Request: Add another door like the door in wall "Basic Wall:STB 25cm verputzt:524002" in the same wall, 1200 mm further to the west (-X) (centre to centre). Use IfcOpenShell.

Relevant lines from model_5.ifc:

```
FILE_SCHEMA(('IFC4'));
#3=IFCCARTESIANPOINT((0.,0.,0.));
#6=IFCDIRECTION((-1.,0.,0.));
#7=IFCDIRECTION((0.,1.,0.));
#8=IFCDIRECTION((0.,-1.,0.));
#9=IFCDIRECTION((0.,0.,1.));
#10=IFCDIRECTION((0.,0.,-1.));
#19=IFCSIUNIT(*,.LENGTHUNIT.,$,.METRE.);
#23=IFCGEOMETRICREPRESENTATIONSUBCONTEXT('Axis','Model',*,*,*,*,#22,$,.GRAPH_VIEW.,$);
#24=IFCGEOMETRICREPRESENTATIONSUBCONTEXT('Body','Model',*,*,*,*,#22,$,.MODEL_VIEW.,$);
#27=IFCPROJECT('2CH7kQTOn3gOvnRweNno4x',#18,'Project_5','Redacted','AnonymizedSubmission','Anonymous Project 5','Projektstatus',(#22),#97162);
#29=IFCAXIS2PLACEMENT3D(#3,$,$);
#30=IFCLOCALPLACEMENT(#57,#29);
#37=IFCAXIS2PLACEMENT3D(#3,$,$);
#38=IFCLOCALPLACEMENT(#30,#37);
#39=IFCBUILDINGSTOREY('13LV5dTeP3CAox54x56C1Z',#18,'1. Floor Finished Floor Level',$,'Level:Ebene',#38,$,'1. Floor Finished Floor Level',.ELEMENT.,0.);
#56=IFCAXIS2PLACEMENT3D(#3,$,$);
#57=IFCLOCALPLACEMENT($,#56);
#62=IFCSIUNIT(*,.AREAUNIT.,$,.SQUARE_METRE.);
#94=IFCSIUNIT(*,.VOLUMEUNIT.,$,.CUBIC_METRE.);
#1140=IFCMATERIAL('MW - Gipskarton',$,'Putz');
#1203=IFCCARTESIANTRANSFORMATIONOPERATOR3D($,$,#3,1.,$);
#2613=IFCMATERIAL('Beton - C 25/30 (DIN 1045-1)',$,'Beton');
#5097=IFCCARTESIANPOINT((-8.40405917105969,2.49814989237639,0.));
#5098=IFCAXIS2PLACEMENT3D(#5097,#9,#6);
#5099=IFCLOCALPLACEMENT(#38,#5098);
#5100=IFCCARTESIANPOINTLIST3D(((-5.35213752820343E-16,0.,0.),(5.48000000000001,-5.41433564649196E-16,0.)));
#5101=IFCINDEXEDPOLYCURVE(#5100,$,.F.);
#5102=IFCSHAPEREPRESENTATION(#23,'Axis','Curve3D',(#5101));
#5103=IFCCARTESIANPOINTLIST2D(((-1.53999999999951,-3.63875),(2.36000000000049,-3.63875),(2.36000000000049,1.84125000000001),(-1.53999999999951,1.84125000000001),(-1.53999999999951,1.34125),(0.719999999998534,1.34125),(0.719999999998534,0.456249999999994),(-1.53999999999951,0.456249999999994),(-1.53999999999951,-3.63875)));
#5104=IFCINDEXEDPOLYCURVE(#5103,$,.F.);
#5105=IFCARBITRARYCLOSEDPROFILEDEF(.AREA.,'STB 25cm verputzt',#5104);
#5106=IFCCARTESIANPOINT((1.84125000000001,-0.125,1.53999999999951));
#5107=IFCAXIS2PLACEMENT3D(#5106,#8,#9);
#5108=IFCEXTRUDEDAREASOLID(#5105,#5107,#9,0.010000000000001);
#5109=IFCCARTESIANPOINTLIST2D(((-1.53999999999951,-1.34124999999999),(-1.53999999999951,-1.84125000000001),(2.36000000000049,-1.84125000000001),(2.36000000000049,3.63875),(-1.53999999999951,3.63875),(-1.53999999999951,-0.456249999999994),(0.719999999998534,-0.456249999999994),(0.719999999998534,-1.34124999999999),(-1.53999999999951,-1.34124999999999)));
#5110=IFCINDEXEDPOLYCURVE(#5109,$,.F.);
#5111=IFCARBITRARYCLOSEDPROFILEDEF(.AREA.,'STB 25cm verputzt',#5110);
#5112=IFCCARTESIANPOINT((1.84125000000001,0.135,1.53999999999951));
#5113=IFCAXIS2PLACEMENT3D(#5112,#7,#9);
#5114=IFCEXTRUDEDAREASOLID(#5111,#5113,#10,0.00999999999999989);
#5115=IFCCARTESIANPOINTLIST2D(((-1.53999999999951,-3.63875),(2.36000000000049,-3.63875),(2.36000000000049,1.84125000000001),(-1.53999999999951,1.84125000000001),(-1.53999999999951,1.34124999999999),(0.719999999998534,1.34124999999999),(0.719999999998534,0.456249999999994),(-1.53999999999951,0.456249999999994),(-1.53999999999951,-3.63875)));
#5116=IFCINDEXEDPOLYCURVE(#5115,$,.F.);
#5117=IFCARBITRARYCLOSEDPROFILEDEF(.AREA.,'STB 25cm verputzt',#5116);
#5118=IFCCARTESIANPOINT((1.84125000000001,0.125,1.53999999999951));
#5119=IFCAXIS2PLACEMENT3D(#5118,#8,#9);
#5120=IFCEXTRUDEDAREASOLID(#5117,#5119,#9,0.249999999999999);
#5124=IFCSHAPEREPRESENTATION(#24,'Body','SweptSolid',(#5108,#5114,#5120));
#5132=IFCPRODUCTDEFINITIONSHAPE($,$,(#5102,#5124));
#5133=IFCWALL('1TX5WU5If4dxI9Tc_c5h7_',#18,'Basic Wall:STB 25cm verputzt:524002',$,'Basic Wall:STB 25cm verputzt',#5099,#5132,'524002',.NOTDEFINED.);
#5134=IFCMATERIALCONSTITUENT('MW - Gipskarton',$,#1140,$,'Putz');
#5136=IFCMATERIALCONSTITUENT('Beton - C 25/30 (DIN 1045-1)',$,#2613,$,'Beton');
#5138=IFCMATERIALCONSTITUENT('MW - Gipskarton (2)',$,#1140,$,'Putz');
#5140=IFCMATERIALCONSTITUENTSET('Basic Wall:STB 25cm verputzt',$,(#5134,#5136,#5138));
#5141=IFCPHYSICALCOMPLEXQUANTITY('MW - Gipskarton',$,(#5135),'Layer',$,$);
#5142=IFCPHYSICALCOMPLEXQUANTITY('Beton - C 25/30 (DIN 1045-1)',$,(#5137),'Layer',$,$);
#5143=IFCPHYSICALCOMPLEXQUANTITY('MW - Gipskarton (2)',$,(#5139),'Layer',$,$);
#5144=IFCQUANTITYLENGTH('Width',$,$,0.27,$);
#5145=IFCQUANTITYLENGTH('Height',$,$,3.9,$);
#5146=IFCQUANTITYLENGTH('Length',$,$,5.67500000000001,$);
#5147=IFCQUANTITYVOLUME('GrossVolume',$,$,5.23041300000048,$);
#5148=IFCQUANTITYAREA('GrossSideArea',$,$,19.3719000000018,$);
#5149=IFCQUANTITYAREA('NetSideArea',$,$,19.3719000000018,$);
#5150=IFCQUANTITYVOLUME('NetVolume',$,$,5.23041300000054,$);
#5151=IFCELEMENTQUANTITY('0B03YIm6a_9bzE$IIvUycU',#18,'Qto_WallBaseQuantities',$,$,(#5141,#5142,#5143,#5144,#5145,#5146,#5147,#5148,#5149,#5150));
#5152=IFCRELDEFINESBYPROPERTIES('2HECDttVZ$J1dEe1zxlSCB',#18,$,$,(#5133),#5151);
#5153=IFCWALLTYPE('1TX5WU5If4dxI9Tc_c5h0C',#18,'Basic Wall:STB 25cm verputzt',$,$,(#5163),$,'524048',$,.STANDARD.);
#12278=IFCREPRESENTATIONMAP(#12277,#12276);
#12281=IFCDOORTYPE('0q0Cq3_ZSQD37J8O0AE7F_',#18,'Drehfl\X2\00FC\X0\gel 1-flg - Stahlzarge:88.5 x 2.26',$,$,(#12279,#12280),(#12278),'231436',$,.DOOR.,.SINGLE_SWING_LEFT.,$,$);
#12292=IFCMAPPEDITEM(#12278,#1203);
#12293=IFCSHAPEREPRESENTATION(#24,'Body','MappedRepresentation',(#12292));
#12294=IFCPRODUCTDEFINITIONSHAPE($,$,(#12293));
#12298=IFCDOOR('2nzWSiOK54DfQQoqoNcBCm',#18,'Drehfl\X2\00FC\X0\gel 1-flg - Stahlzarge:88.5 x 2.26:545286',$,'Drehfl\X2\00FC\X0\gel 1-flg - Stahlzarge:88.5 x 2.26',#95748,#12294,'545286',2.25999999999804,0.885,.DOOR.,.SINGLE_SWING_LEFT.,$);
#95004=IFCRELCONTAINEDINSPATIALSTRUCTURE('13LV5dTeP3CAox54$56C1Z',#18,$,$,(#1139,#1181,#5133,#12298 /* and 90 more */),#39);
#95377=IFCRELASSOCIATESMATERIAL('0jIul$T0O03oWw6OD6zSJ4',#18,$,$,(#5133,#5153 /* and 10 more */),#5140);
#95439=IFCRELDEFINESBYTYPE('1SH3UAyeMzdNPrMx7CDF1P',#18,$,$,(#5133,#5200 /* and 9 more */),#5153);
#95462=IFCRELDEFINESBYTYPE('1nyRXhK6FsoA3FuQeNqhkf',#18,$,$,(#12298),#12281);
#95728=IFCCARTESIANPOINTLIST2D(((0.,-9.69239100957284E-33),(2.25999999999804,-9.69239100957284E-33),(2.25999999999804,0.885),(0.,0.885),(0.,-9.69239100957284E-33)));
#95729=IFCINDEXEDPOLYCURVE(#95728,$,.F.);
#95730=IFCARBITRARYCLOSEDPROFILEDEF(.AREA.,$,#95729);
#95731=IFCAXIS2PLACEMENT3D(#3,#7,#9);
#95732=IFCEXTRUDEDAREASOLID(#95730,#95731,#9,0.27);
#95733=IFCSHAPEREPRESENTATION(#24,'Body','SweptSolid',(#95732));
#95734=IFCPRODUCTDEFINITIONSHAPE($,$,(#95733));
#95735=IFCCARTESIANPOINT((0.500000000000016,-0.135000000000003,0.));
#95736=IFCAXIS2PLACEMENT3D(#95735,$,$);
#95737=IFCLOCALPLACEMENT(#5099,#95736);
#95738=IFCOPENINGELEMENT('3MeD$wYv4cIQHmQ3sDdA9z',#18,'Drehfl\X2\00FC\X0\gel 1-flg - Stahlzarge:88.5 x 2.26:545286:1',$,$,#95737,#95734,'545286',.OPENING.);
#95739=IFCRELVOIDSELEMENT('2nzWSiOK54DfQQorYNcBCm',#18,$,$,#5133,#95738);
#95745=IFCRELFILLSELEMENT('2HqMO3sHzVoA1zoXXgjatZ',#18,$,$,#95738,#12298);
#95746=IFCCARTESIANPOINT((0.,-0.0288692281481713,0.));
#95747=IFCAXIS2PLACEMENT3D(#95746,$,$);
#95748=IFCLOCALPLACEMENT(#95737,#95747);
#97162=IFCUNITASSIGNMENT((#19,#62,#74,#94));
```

```python
import ifcopenshell
import ifcopenshell.api.feature
import ifcopenshell.api.geometry
import ifcopenshell.api.pset
import ifcopenshell.api.root
import ifcopenshell.geom
import ifcopenshell.util.element
import ifcopenshell.util.placement
import ifcopenshell.util.shape
import ifcopenshell.util.unit

model = ifcopenshell.open("model_5.ifc")
unit_scale = ifcopenshell.util.unit.calculate_unit_scale(model)
area_scale = ifcopenshell.util.unit.calculate_unit_scale(model, "AREAUNIT")
volume_scale = ifcopenshell.util.unit.calculate_unit_scale(model, "VOLUMEUNIT")
settings = ifcopenshell.geom.settings()


def volume(element):
    """Net volume in cubic metres, openings subtracted."""
    shape = ifcopenshell.geom.create_shape(settings, element)
    return ifcopenshell.util.shape.get_volume(shape.geometry)


def reuse_history(source, copy):
    """copy_class also copies each property set's owner history, people and application; keep the originals."""
    for rel in copy.IsDefinedBy:
        if rel.is_a("IfcRelDefinesByProperties") and (history := rel.RelatingPropertyDefinition.OwnerHistory):
            rel.RelatingPropertyDefinition.OwnerHistory = source.OwnerHistory
            ifcopenshell.util.element.remove_deep2(model, history)


door = model.by_guid("2nzWSiOK54DfQQoqoNcBCm")
opening = door.FillsVoids[0].RelatingOpeningElement
wall = opening.VoidsElements[0].RelatingBuildingElement
before = volume(wall)
shift = ifcopenshell.util.placement.get_local_placement(wall.ObjectPlacement)[:3, 0] * 1.2 / unit_scale

# copy_class copies the void relationship, type, container and properties, but no geometry.
new_opening = ifcopenshell.api.root.copy_class(model, product=opening)
new_opening.Representation = ifcopenshell.util.element.copy_deep(
    model, opening.Representation, exclude=["IfcGeometricRepresentationContext", "IfcRepresentationMap"]
)
new_opening.Name = "Drehflügel 1-flg - Stahlzarge:88.5 x 2.26"
new_opening.Tag = None
reuse_history(opening, new_opening)
new_door = ifcopenshell.api.root.copy_class(model, product=door)
new_door.Representation = ifcopenshell.util.element.copy_deep(
    model, door.Representation, exclude=["IfcGeometricRepresentationContext", "IfcRepresentationMap"]
)
new_door.Name = "Drehflügel 1-flg - Stahlzarge:88.5 x 2.26"
new_door.Tag = None
reuse_history(door, new_door)
ifcopenshell.api.feature.add_filling(model, opening=new_opening, element=new_door)

for old, new in ((opening, new_opening), (door, new_door)):
    matrix = ifcopenshell.util.placement.get_local_placement(old.ObjectPlacement)
    matrix[:3, 3] += shift
    ifcopenshell.api.geometry.edit_object_placement(model, product=new, matrix=matrix, is_si=False)

after = volume(wall)
thickness = 0.27  # wall thickness in metres

# Update the wall's stored quantities.
qto = model.by_id(ifcopenshell.util.element.get_pset(wall, "Qto_WallBaseQuantities", should_inherit=False)["id"])
ifcopenshell.api.pset.edit_qto(model, qto=qto, properties={
    "NetSideArea": after / thickness / area_scale,
    "NetVolume": after / volume_scale,
})

print(f"wall volume {before:.3f} -> {after:.3f} m3")

model.write("model_5_updated.ifc")
```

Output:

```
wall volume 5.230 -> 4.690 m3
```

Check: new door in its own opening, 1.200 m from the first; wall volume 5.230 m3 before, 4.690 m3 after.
